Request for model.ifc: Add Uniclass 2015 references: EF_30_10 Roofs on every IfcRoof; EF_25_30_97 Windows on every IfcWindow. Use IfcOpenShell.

First a look at what the model holds.

```python
import ifcopenshell

model = ifcopenshell.open("model.ifc")
print(model.schema)
print("classifications:", [c.Name for c in model.by_type("IfcClassification")])
for ifc_class in ("IfcDoor", "IfcRoof", "IfcStair", "IfcWall", "IfcWindow"):
    print(ifc_class, len(model.by_type(ifc_class)))
```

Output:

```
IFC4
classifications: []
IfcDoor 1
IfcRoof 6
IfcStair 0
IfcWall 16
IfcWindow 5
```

```python
import ifcopenshell
import ifcopenshell.api.classification

model = ifcopenshell.open("model.ifc")

system = ifcopenshell.api.classification.add_classification(model, classification="Uniclass 2015")

codes = {
    "IfcRoof": ("EF_30_10", "Roofs"),
    "IfcWindow": ("EF_25_30_97", "Windows"),
}
for ifc_class, (code, name) in codes.items():
    products = model.by_type(ifc_class)
    ifcopenshell.api.classification.add_reference(
        model, products=products, classification=system, identification=code, name=name
    )
    print(code, len(products))

model.write("model_edited.ifc")
```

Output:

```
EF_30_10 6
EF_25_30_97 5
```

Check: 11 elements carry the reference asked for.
